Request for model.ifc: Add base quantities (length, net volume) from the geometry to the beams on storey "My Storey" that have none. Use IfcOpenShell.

First a look at what the model holds.

```python
import ifcopenshell
import ifcopenshell.util.element
import ifcopenshell.util.unit

model = ifcopenshell.open("model.ifc")
print(model.schema)
for unit_type in ("LENGTHUNIT", "AREAUNIT", "VOLUMEUNIT"):
    print(unit_type, ifcopenshell.util.unit.calculate_unit_scale(model, unit_type))
storey = next(s for s in model.by_type("IfcBuildingStorey") if s.Name == "My Storey")
beams = [e for e in ifcopenshell.util.element.get_decomposition(storey) if e.is_a("IfcBeam")]
for e in sorted(beams, key=lambda e: e.id()):
    print(e.id(), e.is_a(), e.Name, list(ifcopenshell.util.element.get_psets(e, qtos_only=True)), sep=" | ")
```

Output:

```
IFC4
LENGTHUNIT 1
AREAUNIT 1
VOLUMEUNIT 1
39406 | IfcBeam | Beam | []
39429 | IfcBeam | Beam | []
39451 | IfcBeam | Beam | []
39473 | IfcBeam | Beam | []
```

```python
import ifcopenshell
import ifcopenshell.api.pset
import ifcopenshell.geom
import ifcopenshell.util.element
import ifcopenshell.util.shape
import ifcopenshell.util.unit

model = ifcopenshell.open("model.ifc")
unit_scale = ifcopenshell.util.unit.calculate_unit_scale(model)
volume_scale = ifcopenshell.util.unit.calculate_unit_scale(model, "VOLUMEUNIT")
settings = ifcopenshell.geom.settings()

storey = next(s for s in model.by_type("IfcBuildingStorey") if s.Name == "My Storey")
beams = [e for e in ifcopenshell.util.element.get_decomposition(storey) if e.is_a("IfcBeam")]

for e in sorted(beams, key=lambda e: e.id()):
    if ifcopenshell.util.element.get_psets(e, qtos_only=True, should_inherit=False):
        continue
    # Geometry comes back in metres, in the element's own axes.
    shape = ifcopenshell.geom.create_shape(settings, e)
    values = {
        "Length": ifcopenshell.util.shape.get_max_xyz(shape.geometry) / unit_scale,
        "NetVolume": ifcopenshell.util.shape.get_volume(shape.geometry) / volume_scale,
    }
    qto = ifcopenshell.api.pset.add_qto(model, product=e, name="Qto_BeamBaseQuantities")
    ifcopenshell.api.pset.edit_qto(model, qto=qto, properties=values)
    print(e.id(), {k: round(v, 3) for k, v in values.items()})

model.write("model-out.ifc")
```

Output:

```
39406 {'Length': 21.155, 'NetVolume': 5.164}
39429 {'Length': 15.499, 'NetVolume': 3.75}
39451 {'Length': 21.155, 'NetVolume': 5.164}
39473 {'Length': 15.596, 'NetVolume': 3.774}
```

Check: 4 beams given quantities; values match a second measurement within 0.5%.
